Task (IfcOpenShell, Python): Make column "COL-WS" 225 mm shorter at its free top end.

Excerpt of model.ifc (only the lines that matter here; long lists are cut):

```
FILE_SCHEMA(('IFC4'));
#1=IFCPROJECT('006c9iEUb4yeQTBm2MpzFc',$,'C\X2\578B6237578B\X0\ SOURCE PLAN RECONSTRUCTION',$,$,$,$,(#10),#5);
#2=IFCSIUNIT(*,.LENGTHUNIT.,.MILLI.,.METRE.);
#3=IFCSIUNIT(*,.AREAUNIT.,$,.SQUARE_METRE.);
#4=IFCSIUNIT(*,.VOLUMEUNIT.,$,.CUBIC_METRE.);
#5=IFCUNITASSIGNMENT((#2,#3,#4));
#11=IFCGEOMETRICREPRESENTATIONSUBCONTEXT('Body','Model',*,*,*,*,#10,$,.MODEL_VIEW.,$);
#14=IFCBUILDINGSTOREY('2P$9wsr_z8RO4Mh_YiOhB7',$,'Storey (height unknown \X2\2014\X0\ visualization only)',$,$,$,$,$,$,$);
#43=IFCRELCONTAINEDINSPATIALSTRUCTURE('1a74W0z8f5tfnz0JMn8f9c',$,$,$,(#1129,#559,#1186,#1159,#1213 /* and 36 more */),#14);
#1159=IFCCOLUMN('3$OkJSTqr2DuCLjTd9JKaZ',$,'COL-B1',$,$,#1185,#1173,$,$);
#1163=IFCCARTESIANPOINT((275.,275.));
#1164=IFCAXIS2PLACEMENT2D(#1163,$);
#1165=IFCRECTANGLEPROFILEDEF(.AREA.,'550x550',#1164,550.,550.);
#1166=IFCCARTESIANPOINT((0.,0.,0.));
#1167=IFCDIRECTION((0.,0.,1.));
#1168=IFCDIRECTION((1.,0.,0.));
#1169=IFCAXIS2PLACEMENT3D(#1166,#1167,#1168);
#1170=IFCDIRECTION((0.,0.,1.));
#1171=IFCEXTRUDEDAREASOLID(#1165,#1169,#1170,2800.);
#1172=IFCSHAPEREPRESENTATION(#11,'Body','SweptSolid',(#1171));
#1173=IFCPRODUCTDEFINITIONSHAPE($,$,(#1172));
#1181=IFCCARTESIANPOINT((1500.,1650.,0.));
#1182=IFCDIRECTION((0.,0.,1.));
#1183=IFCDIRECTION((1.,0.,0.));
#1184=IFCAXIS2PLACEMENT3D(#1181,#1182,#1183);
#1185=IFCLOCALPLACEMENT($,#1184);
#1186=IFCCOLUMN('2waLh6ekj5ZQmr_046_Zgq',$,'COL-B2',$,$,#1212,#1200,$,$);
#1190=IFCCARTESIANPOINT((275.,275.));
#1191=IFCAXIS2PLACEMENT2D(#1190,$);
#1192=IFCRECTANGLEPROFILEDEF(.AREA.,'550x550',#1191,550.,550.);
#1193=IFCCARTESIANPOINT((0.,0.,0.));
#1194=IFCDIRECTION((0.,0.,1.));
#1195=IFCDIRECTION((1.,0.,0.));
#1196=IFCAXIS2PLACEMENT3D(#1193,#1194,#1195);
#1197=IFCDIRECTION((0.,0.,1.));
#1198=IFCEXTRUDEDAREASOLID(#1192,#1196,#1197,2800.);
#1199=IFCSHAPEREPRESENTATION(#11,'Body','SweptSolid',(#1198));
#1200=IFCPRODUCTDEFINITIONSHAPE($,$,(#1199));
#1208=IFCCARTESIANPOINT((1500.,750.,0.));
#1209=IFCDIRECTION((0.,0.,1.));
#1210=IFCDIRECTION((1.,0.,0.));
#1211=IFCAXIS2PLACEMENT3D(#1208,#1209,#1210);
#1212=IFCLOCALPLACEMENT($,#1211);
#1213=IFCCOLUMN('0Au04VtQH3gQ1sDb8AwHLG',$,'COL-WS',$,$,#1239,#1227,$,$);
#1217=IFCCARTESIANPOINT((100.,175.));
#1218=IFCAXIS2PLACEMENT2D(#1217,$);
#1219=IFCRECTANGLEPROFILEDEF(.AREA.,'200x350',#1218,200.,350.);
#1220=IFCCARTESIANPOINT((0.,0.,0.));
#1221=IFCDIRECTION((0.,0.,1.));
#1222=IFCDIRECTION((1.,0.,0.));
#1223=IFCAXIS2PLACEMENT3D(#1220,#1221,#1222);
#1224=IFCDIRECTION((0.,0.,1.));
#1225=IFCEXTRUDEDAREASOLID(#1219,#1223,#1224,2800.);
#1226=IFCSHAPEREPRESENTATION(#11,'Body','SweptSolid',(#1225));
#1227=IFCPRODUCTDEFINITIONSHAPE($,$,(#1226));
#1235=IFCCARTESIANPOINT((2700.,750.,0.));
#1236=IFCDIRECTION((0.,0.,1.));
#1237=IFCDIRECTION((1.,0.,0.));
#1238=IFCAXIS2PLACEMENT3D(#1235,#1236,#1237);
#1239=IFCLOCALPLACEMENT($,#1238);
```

```python
import ifcopenshell
import ifcopenshell.util.representation

model = ifcopenshell.open("model.ifc")

member = model.by_guid("0Au04VtQH3gQ1sDb8AwHLG")
change = -225.0

# The extrusion runs towards the end named, so only its depth changes.
body = ifcopenshell.util.representation.get_representation(member, "Model", "Body")
solid = body.Items[0]
old_length = solid.Depth
solid.Depth += change

print(f"length {old_length:g} -> {solid.Depth:g}")

model.write("model-out.ifc")
```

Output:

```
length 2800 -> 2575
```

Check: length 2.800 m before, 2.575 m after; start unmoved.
